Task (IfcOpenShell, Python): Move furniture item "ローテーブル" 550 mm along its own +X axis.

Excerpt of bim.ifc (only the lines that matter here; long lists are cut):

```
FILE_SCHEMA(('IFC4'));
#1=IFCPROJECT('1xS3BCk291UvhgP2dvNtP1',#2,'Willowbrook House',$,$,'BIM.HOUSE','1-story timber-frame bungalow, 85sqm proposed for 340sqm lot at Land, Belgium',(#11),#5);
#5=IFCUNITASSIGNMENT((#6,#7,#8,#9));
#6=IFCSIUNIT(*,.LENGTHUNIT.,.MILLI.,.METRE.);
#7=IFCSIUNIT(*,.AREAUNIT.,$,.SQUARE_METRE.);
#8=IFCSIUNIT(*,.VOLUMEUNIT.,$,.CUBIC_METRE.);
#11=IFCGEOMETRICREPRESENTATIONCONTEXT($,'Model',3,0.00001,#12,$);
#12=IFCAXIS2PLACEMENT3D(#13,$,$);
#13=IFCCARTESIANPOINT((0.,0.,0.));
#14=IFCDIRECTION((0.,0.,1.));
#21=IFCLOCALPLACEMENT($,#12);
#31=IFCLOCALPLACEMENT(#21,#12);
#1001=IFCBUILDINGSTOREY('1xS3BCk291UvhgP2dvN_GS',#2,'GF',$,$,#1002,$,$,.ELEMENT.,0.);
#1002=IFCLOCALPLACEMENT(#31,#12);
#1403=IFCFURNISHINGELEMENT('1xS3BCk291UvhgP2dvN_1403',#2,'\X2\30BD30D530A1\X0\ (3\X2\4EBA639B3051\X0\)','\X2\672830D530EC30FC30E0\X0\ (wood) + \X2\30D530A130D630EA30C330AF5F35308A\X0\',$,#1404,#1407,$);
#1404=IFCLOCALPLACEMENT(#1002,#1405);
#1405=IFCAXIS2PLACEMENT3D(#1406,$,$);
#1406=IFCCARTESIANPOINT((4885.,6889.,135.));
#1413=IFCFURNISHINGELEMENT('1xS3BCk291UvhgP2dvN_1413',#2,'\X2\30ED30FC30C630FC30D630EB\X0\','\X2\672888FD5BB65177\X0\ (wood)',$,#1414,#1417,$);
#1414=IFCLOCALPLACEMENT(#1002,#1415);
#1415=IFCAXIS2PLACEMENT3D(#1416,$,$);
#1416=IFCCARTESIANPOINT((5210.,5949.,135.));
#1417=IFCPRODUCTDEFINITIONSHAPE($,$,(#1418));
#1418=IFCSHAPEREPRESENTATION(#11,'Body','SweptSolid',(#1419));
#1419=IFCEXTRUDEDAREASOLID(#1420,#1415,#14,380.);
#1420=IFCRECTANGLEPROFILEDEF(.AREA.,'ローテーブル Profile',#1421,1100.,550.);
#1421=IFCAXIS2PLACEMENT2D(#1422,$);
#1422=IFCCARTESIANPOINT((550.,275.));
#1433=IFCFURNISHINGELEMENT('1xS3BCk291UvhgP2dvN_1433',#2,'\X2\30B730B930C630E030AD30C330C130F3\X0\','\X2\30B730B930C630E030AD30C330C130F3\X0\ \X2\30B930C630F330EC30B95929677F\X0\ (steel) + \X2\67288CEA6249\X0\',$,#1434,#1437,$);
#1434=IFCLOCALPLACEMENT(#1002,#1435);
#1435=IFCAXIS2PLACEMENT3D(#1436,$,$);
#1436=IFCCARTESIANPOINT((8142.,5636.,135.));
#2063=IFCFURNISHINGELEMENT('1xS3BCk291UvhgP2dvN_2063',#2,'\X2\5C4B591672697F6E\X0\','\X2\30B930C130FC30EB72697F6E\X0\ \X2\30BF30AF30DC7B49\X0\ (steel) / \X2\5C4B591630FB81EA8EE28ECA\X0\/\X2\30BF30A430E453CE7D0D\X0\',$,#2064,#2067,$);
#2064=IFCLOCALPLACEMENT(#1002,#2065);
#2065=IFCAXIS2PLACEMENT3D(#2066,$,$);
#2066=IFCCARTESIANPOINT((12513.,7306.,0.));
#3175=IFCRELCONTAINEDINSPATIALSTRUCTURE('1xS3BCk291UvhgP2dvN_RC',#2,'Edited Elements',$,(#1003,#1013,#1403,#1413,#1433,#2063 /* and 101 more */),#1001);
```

```python
import ifcopenshell
import ifcopenshell.api.geometry
import ifcopenshell.util.placement

model = ifcopenshell.open("bim.ifc")

item = model.by_id(1413)
matrix = ifcopenshell.util.placement.get_local_placement(item.ObjectPlacement)
matrix[:3, 3] += matrix[:3, 0] * 550.0
ifcopenshell.api.geometry.edit_object_placement(model, product=item, matrix=matrix, is_si=False)

print(ifcopenshell.util.placement.get_local_placement(item.ObjectPlacement).round(3) + 0.0)

model.write("bim-out.ifc")
```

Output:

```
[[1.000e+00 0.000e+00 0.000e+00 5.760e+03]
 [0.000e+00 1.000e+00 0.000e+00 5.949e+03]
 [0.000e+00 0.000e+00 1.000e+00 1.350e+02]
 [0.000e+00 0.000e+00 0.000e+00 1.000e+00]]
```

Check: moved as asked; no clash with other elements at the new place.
